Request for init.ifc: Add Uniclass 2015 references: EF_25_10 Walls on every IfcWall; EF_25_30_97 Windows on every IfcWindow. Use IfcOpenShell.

First a look at what the model holds.

```python
import ifcopenshell

model = ifcopenshell.open("init.ifc")
print(model.schema)
print("classifications:", [c.Name for c in model.by_type("IfcClassification")])
for ifc_class in ("IfcDoor", "IfcRoof", "IfcStair", "IfcWall", "IfcWindow"):
    print(ifc_class, len(model.by_type(ifc_class)))
```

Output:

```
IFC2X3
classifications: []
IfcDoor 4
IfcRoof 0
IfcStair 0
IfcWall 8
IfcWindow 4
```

```python
import ifcopenshell
import ifcopenshell.api.classification

model = ifcopenshell.open("init.ifc")

# IFC2X3 requires Source and Edition and has no link from the project to the system.
system = model.create_entity("IfcClassification", Source="NBS", Edition="2015", Name="Uniclass 2015")

codes = {
    "IfcWall": ("EF_25_10", "Walls"),
    "IfcWindow": ("EF_25_30_97", "Windows"),
}
for ifc_class, (code, name) in codes.items():
    products = model.by_type(ifc_class)
    ifcopenshell.api.classification.add_reference(
        model, products=products, classification=system, identification=code, name=name
    )
    print(code, len(products))

model.write("init_v2.ifc")
```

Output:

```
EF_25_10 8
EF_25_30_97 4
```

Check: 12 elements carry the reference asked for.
